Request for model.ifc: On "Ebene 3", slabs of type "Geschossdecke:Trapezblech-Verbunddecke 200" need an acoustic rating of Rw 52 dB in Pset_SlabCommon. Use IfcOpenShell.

First a look at what the model holds.

```python
import ifcopenshell
import ifcopenshell.util.element

model = ifcopenshell.open("model.ifc")
print(model.schema)
storey = next(s for s in model.by_type("IfcBuildingStorey") if s.Name == "Ebene 3")
slabs = [e for e in ifcopenshell.util.element.get_decomposition(storey) if e.is_a("IfcSlab")]
seen = {}
for e in slabs:
    element_type = ifcopenshell.util.element.get_type(e)
    key = (element_type.Name if element_type != e and element_type else None, ifcopenshell.util.element.get_pset(e, "Pset_SlabCommon", "AcousticRating"))
    seen[key] = seen.get(key, 0) + 1
for (name, value), count in sorted(seen.items(), key=str):
    print(count, "x", name, "|", value)
```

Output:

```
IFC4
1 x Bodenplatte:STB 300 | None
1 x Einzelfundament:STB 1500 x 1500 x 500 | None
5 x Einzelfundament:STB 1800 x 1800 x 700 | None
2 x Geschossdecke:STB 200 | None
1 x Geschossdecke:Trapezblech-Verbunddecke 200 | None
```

```python
import ifcopenshell
import ifcopenshell.api.pset
import ifcopenshell.util.element

model = ifcopenshell.open("model.ifc")

storey = next(s for s in model.by_type("IfcBuildingStorey") if s.Name == "Ebene 3")
slabs = [e for e in ifcopenshell.util.element.get_decomposition(storey) if e.is_a("IfcSlab")]

count = 0
for e in slabs:
    element_type = ifcopenshell.util.element.get_type(e)
    if element_type in (None, e) or element_type.Name != "Geschossdecke:Trapezblech-Verbunddecke 200":
        continue
    # add_pset returns the element's existing set when there is one.
    pset = ifcopenshell.api.pset.add_pset(model, product=e, name="Pset_SlabCommon")
    ifcopenshell.api.pset.edit_pset(model, pset=pset, properties={"AcousticRating": "Rw 52 dB"})
    count += 1

print(count, "slabs updated")

model.write("model-out.ifc")
```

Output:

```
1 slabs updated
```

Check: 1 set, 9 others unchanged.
